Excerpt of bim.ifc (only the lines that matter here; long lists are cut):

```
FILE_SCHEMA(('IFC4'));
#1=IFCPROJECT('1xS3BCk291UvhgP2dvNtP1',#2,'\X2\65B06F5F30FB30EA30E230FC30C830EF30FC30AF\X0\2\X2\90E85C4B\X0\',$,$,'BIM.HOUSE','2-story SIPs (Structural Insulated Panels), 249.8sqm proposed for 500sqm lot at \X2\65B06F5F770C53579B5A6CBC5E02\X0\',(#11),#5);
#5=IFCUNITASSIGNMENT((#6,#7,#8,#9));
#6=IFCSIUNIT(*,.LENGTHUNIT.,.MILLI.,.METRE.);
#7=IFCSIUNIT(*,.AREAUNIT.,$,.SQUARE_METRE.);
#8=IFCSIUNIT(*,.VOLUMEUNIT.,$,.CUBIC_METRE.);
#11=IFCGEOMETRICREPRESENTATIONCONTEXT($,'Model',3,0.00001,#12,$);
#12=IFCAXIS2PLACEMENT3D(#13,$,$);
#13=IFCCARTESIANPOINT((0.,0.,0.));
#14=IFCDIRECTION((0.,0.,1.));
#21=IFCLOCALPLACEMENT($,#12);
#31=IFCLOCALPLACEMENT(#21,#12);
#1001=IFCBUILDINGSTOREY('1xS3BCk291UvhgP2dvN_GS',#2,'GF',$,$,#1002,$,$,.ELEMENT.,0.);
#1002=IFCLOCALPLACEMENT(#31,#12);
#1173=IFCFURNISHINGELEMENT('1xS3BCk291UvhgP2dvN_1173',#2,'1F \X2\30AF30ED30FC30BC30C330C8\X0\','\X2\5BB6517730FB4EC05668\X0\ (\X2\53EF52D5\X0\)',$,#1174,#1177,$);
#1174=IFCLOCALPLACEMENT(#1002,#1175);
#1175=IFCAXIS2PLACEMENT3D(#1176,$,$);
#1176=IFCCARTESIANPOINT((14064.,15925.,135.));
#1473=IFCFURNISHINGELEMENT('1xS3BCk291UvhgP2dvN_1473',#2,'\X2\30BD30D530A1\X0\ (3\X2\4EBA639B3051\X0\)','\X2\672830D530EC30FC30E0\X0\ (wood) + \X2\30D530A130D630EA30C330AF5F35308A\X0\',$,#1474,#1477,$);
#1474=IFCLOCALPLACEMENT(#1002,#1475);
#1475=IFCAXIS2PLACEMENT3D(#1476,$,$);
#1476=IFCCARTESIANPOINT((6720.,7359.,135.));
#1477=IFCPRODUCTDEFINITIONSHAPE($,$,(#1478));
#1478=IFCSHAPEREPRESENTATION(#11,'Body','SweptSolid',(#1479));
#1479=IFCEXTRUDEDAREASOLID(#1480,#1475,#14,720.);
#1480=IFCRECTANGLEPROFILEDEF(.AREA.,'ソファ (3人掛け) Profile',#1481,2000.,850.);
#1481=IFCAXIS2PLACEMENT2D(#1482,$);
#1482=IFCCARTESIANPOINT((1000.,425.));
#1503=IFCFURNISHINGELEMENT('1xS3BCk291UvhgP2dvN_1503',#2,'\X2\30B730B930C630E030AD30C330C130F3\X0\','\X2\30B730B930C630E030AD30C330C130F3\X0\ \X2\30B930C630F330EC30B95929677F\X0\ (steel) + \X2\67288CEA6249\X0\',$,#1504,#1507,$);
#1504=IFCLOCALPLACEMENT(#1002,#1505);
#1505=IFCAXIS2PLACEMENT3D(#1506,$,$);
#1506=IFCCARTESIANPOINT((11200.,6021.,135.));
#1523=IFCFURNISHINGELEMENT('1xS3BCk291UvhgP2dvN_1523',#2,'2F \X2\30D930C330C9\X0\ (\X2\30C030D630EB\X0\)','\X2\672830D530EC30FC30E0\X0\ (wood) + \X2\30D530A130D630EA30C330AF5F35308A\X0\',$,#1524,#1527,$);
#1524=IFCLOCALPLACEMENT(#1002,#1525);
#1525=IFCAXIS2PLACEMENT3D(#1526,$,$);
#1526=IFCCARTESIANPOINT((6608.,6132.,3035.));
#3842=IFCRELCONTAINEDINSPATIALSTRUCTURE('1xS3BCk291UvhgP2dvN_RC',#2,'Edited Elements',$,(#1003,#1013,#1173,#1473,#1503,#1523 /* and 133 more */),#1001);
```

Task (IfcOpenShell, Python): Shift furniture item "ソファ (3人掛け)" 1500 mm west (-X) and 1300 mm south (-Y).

```python
import ifcopenshell
import ifcopenshell.api.geometry
import ifcopenshell.util.placement

model = ifcopenshell.open("bim.ifc")

item = model.by_id(1473)
matrix = ifcopenshell.util.placement.get_local_placement(item.ObjectPlacement)
matrix[0, 3] -= 1500.0
matrix[1, 3] -= 1300.0
ifcopenshell.api.geometry.edit_object_placement(model, product=item, matrix=matrix, is_si=False)

print(ifcopenshell.util.placement.get_local_placement(item.ObjectPlacement).round(3) + 0.0)

model.write("bim_rev.ifc")
```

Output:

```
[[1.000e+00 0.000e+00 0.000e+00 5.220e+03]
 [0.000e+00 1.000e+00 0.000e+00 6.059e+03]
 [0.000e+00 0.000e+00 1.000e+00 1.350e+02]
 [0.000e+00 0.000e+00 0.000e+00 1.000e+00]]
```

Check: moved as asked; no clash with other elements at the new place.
